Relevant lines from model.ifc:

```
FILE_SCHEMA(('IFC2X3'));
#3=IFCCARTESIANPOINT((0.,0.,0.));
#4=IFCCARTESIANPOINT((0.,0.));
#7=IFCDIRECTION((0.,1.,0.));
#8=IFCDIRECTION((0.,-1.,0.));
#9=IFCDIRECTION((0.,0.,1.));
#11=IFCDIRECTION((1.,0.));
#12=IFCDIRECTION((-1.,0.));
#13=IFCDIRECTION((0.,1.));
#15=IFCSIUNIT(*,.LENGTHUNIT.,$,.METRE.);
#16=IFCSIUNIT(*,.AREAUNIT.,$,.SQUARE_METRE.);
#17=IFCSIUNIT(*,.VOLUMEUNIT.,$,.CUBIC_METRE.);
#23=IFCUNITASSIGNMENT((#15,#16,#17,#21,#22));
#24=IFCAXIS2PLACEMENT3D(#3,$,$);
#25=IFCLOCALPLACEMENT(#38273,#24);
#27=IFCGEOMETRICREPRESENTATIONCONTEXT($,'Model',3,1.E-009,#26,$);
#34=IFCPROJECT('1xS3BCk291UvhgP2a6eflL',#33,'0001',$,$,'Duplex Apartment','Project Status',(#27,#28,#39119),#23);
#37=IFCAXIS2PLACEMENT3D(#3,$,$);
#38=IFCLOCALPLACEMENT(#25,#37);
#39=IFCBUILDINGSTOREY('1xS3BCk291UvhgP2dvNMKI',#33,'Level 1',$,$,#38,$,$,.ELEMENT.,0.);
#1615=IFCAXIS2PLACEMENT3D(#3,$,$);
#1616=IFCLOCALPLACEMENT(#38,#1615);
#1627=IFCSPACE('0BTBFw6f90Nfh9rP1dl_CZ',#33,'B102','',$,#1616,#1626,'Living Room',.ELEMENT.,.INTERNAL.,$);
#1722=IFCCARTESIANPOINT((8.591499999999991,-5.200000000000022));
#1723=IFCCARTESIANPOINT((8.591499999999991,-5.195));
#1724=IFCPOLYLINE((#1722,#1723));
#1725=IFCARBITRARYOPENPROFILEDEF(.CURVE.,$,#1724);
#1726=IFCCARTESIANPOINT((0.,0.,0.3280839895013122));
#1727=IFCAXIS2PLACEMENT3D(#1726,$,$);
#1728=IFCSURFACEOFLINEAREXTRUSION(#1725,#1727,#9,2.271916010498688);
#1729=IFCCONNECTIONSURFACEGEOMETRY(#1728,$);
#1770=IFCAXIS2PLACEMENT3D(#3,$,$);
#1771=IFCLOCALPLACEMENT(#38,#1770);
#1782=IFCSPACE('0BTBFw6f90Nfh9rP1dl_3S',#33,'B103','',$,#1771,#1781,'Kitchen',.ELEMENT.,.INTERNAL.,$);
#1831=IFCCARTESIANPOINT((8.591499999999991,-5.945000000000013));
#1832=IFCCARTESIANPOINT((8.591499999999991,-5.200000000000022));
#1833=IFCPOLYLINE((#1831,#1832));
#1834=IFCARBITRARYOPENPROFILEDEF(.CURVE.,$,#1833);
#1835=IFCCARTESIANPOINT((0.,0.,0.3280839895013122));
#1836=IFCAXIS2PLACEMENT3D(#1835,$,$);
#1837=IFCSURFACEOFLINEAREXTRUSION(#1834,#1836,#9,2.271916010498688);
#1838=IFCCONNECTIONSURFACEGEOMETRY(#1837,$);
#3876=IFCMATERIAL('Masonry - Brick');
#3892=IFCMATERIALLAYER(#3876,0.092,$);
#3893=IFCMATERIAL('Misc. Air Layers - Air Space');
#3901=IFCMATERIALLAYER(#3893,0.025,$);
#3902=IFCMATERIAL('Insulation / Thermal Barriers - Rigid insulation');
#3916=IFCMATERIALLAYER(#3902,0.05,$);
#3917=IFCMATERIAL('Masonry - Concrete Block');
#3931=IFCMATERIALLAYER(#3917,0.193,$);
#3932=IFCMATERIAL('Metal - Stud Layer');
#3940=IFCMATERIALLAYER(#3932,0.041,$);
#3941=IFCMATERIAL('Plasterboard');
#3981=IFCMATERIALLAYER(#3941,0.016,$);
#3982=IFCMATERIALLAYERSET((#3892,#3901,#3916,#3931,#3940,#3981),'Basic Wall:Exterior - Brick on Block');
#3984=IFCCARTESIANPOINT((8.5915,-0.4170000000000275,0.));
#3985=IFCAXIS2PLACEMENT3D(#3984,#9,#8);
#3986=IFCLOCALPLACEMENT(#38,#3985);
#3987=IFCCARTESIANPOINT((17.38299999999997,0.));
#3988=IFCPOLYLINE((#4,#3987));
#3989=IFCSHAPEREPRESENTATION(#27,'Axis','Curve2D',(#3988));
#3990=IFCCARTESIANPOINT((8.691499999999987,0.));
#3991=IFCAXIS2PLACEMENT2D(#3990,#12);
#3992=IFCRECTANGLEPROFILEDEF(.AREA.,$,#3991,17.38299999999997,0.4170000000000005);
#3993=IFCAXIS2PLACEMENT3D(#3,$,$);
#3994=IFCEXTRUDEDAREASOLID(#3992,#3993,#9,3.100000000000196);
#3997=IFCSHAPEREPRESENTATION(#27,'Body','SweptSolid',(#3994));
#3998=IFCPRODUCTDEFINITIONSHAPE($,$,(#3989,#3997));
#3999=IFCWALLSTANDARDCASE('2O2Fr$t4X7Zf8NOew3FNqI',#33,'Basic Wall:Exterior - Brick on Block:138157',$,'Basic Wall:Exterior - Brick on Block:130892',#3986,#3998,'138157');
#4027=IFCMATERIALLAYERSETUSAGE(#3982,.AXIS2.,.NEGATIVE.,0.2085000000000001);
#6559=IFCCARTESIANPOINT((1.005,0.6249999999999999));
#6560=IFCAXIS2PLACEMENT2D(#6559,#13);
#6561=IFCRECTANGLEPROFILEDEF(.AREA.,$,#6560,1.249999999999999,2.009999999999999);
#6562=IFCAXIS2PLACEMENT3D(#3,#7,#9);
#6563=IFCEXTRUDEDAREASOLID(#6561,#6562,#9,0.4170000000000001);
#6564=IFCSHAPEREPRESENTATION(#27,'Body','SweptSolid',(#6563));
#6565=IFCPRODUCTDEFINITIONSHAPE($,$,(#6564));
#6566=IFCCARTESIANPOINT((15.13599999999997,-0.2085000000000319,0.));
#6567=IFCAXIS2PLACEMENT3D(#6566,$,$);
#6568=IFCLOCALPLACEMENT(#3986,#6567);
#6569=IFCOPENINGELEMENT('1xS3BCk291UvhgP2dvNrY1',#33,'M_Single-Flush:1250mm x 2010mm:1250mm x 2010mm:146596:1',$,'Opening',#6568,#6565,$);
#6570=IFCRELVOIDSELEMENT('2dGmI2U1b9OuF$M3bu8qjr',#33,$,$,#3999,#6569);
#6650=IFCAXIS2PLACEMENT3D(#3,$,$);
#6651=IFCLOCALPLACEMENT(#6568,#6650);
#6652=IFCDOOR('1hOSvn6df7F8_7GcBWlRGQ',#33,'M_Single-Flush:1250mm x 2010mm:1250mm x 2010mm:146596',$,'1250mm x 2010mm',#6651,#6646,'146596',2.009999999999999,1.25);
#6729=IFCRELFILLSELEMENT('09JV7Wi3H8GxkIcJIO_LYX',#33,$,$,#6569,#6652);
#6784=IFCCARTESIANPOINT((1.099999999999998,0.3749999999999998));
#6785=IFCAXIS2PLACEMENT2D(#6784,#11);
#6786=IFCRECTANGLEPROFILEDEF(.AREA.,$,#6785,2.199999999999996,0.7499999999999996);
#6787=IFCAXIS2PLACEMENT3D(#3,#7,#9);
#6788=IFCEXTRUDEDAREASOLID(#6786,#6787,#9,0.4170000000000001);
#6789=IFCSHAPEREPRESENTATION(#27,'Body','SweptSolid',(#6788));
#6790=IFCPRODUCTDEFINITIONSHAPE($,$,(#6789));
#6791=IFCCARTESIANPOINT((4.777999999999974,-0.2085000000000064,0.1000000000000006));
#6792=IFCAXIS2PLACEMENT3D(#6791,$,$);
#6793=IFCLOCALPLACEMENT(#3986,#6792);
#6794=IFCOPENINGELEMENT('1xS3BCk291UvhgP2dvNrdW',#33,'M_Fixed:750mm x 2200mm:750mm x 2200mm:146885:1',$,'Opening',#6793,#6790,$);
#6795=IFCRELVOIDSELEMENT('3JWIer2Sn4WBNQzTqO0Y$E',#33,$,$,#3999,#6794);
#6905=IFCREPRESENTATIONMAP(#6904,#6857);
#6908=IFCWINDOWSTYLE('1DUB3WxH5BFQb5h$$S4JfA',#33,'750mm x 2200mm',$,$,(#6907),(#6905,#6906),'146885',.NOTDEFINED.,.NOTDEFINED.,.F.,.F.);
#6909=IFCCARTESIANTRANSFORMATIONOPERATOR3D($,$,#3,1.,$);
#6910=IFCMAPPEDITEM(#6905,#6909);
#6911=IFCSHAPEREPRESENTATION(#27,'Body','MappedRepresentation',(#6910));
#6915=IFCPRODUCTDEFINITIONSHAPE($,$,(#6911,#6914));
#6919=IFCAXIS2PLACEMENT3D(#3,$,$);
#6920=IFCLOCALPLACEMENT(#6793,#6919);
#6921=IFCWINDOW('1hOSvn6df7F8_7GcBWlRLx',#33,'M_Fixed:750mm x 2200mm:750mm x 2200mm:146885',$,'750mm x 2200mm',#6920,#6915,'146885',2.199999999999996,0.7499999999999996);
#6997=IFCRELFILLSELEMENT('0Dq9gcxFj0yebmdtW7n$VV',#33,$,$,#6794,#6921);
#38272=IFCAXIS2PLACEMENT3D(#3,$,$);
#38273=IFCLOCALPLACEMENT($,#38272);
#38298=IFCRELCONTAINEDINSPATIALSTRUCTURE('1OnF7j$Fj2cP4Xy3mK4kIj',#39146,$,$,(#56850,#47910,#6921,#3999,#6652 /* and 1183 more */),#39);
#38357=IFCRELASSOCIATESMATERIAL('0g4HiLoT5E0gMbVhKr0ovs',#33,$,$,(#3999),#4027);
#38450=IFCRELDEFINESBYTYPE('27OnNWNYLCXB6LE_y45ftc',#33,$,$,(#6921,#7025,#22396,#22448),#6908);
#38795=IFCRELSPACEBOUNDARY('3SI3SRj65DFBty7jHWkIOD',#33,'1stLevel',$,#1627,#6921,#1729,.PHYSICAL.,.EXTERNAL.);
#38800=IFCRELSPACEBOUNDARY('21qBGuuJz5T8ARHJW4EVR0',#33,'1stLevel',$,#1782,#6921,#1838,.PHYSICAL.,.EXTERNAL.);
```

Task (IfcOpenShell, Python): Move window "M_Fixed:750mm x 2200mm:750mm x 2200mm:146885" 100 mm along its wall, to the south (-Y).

```python
import numpy as np
import ifcopenshell
import ifcopenshell.api.geometry
import ifcopenshell.util.placement
import ifcopenshell.util.unit

model = ifcopenshell.open("model.ifc")
unit_scale = ifcopenshell.util.unit.calculate_unit_scale(model)

window = model.by_guid("1hOSvn6df7F8_7GcBWlRLx")
opening = window.FillsVoids[0].RelatingOpeningElement
wall = opening.VoidsElements[0].RelatingBuildingElement

wall_matrix = ifcopenshell.util.placement.get_local_placement(wall.ObjectPlacement)
shift = wall_matrix[:3, 0] * 0.1 / unit_scale
before = ifcopenshell.util.placement.get_local_placement(window.ObjectPlacement)[:3, 3].copy()

# The window is placed relative to its opening, so it follows when the opening moves.
matrix = ifcopenshell.util.placement.get_local_placement(opening.ObjectPlacement)
matrix[:3, 3] += shift
ifcopenshell.api.geometry.edit_object_placement(
    model, product=opening, matrix=matrix, is_si=False, should_transform_children=True
)

# Space boundary surfaces are stored in each space's coordinates; move them too.
for rel in window.ProvidesBoundaries:
    if not rel.ConnectionGeometry:
        continue
    surface = rel.ConnectionGeometry.SurfaceOnRelatingElement
    space_matrix = ifcopenshell.util.placement.get_local_placement(rel.RelatingSpace.ObjectPlacement)
    point = np.array(surface.Position.Location.Coordinates) + space_matrix[:3, :3].T @ shift
    surface.Position = model.createIfcAxis2Placement3D(
        model.createIfcCartesianPoint(point.tolist()), surface.Position.Axis, surface.Position.RefDirection
    )

after = ifcopenshell.util.placement.get_local_placement(window.ObjectPlacement)[:3, 3]
print("window moved by", (after - before).round(3) + 0.0)

model.write("model_v2.ifc")
```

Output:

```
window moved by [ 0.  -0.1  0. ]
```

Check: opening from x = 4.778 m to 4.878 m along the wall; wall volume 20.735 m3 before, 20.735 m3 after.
